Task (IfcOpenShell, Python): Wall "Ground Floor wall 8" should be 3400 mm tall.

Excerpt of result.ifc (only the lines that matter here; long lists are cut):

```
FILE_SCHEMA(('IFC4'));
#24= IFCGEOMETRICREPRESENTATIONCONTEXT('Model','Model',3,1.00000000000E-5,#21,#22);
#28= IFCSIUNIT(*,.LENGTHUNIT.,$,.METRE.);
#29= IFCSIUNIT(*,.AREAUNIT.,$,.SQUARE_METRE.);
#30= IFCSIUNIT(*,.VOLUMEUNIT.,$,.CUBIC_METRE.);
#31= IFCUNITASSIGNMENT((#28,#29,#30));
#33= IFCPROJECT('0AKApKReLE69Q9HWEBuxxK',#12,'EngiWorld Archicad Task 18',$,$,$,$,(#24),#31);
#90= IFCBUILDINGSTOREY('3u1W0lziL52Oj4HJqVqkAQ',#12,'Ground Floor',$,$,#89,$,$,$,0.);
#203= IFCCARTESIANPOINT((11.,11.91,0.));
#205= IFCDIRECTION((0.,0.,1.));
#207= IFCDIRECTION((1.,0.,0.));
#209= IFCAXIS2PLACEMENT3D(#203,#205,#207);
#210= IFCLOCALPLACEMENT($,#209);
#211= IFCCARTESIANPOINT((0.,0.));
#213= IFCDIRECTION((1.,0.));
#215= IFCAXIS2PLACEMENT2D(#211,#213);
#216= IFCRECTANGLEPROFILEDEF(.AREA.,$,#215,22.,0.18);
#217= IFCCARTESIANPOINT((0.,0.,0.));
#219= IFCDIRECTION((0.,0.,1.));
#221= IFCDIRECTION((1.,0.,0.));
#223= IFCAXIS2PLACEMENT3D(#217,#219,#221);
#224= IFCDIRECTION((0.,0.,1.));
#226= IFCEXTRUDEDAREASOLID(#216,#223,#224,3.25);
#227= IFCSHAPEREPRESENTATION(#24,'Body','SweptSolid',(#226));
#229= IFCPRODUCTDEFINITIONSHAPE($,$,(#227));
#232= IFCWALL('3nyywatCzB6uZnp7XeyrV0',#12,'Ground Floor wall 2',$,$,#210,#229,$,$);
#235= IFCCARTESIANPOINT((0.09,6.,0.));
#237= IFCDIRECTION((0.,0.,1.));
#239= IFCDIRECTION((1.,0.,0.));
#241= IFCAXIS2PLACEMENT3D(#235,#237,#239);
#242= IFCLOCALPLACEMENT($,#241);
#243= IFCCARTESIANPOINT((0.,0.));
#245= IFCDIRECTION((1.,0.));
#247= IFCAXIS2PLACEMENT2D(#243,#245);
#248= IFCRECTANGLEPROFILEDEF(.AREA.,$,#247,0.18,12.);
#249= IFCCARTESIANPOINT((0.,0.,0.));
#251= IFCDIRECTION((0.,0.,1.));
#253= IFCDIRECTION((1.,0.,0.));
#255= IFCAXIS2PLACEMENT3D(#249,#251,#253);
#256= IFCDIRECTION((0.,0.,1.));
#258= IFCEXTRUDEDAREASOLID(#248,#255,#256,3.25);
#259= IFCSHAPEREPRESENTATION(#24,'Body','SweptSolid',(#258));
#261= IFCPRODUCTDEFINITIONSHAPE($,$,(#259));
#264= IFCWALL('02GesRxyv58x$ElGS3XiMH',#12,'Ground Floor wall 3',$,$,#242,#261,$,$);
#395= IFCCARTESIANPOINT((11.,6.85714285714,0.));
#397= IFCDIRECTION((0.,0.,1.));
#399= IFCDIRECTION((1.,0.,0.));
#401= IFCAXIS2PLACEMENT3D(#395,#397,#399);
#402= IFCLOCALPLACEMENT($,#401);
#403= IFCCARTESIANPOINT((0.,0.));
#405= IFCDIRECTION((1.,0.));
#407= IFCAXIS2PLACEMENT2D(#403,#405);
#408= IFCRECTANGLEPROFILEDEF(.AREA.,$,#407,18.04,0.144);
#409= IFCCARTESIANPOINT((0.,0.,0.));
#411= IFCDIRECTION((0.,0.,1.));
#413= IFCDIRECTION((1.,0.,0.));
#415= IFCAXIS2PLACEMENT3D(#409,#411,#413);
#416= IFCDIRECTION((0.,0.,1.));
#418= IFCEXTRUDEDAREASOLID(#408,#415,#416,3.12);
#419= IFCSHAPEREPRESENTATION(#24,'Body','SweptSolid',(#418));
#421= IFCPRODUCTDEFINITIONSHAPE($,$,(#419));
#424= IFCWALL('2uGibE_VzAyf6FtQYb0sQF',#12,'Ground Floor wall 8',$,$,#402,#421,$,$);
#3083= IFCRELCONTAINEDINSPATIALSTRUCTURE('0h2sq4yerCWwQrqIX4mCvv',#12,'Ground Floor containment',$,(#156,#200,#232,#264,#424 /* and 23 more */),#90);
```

```python
import ifcopenshell
import ifcopenshell.geom
import ifcopenshell.util.shape
import ifcopenshell.util.unit

model = ifcopenshell.open("result.ifc")
unit_scale = ifcopenshell.util.unit.calculate_unit_scale(model)
settings = ifcopenshell.geom.settings()


def volume(element):
    """Net volume in cubic metres, openings subtracted."""
    shape = ifcopenshell.geom.create_shape(settings, element)
    return ifcopenshell.util.shape.get_volume(shape.geometry)


wall = model.by_guid("2uGibE_VzAyf6FtQYb0sQF")
before = volume(wall)

body = next(r for r in wall.Representation.Representations if r.RepresentationIdentifier == "Body")
solid = body.Items[0]
old_height = solid.Depth
solid.Depth = 3.4 / unit_scale
after = volume(wall)

print(f"height {old_height:g} -> {solid.Depth:g}, volume {before:.3f} -> {after:.3f} m3")

model.write("result_updated.ifc")
```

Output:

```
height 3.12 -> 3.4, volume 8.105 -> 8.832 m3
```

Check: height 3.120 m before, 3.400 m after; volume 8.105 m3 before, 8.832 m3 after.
